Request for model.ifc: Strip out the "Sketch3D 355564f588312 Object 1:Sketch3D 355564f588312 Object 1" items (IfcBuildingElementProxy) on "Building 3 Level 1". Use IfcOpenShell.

First a look at what the model holds.

```python
import ifcopenshell
import ifcopenshell.util.element

model = ifcopenshell.open("model.ifc")
print(model.schema)
storey = next(s for s in model.by_type("IfcBuildingStorey") if s.Name == "Building 3 Level 1")
proxies = [e for e in ifcopenshell.util.element.get_decomposition(storey) if e.is_a("IfcBuildingElementProxy")]
seen = {}
for e in proxies:
    element_type = ifcopenshell.util.element.get_type(e)
    name = element_type.Name if element_type not in (None, e) else None
    seen[name] = seen.get(name, 0) + 1
for name, count in sorted(seen.items(), key=str):
    print(count, "x", name)
```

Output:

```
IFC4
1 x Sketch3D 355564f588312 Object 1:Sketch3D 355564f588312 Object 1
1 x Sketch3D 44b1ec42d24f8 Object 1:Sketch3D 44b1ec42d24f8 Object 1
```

```python
import ifcopenshell
import ifcopenshell.api.root
import ifcopenshell.util.element

model = ifcopenshell.open("model.ifc")

storey = next(s for s in model.by_type("IfcBuildingStorey") if s.Name == "Building 3 Level 1")
proxies = [e for e in ifcopenshell.util.element.get_decomposition(storey) if e.is_a("IfcBuildingElementProxy")]
targets = [e for e in proxies if (t := ifcopenshell.util.element.get_type(e)) not in (None, e) and t.Name == "Sketch3D 355564f588312 Object 1:Sketch3D 355564f588312 Object 1"]

for e in targets:
    ifcopenshell.api.root.remove_product(model, product=e)
print(len(targets), "removed")

model.write("model_v2.ifc")
```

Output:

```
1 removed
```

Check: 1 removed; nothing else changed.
